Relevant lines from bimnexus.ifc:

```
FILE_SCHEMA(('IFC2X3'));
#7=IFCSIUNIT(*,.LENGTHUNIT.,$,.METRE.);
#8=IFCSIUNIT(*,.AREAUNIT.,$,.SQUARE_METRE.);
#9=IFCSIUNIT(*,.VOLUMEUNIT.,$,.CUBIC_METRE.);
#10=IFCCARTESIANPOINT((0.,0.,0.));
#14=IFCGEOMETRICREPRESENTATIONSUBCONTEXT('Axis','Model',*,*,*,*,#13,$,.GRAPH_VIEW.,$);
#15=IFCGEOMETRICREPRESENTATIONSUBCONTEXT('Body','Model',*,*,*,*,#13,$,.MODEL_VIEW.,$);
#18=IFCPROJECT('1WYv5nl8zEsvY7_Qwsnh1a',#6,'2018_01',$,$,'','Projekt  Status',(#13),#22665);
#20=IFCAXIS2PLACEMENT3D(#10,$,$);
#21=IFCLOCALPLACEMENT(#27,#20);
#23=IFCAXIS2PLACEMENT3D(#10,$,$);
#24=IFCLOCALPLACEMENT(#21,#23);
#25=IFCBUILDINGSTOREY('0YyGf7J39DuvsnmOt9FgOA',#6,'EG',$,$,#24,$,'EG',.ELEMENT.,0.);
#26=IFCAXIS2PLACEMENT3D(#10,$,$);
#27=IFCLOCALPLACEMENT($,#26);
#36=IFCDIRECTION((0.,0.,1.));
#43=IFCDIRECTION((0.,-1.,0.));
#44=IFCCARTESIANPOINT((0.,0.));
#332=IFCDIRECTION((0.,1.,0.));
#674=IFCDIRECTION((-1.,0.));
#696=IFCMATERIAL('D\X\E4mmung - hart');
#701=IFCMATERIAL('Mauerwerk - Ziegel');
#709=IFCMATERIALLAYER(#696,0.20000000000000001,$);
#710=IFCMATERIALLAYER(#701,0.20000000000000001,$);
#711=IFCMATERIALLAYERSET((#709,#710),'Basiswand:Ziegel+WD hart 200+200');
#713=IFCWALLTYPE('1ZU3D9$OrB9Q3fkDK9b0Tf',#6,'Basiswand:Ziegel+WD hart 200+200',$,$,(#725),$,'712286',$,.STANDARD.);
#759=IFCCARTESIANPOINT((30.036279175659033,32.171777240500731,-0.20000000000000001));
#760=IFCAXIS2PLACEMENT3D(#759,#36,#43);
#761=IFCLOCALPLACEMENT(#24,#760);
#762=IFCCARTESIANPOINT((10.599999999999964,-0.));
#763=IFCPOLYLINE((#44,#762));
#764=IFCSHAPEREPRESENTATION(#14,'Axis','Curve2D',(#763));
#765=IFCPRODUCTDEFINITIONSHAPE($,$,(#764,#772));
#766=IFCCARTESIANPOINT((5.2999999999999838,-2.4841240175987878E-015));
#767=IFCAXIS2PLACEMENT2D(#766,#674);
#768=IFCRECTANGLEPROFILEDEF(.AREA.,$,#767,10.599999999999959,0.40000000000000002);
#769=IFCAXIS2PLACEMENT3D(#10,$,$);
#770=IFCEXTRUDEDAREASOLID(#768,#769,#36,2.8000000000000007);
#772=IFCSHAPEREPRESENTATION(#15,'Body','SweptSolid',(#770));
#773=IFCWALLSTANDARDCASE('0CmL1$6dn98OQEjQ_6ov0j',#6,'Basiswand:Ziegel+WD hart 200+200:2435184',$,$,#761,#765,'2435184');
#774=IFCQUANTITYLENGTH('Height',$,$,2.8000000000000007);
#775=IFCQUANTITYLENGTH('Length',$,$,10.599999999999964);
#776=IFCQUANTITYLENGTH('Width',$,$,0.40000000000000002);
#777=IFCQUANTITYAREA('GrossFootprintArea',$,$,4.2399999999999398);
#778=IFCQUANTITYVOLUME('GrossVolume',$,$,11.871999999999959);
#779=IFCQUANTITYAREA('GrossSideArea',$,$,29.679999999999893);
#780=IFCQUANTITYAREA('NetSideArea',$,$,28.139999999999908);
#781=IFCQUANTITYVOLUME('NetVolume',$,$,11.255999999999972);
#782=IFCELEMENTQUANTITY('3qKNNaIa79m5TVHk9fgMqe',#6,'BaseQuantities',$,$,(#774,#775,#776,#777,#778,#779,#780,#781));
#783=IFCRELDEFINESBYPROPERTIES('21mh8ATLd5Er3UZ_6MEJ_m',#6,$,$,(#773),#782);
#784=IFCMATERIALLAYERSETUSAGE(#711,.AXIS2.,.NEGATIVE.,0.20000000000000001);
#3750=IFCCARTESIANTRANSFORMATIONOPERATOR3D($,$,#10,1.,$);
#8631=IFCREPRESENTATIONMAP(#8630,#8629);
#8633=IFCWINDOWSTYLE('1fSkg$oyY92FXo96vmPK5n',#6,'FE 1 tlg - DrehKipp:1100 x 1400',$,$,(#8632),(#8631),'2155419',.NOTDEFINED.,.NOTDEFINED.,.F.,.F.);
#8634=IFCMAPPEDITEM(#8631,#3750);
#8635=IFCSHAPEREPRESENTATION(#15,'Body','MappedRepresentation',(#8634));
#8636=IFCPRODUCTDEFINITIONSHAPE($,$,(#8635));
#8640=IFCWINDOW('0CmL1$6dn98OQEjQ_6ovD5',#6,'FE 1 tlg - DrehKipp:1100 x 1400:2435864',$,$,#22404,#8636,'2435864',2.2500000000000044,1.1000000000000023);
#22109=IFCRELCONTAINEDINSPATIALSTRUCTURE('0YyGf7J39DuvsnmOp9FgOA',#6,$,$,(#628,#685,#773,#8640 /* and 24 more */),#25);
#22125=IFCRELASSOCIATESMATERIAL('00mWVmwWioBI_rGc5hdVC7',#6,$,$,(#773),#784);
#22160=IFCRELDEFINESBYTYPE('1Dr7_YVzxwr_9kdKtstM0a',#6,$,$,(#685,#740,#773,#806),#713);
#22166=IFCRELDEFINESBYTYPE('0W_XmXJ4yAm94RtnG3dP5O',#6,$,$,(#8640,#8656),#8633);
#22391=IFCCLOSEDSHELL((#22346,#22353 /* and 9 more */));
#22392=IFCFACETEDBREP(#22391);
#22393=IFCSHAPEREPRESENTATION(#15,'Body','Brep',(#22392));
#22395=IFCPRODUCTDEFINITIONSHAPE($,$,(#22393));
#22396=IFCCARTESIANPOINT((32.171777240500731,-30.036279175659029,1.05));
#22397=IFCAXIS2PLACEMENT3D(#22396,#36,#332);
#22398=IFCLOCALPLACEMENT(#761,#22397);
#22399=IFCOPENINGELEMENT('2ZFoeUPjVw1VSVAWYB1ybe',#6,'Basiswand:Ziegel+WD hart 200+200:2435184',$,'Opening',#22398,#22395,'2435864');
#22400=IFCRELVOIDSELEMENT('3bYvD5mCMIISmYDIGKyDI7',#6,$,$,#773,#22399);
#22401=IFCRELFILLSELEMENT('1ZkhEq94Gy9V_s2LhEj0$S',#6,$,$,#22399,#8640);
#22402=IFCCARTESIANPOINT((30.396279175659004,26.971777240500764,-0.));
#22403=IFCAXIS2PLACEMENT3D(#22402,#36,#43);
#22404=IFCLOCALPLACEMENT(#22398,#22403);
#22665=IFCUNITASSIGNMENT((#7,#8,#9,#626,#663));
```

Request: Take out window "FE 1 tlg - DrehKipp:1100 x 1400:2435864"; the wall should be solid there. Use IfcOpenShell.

```python
import ifcopenshell
import ifcopenshell.api.feature
import ifcopenshell.api.pset
import ifcopenshell.api.root
import ifcopenshell.geom
import ifcopenshell.util.element
import ifcopenshell.util.shape
import ifcopenshell.util.unit

model = ifcopenshell.open("bimnexus.ifc")
area_scale = ifcopenshell.util.unit.calculate_unit_scale(model, "AREAUNIT")
volume_scale = ifcopenshell.util.unit.calculate_unit_scale(model, "VOLUMEUNIT")
settings = ifcopenshell.geom.settings()


def volume(element):
    """Net volume in cubic metres, openings subtracted."""
    shape = ifcopenshell.geom.create_shape(settings, element)
    return ifcopenshell.util.shape.get_volume(shape.geometry)


window = model.by_guid("0CmL1$6dn98OQEjQ_6ovD5")
opening = window.FillsVoids[0].RelatingOpeningElement
wall = opening.VoidsElements[0].RelatingBuildingElement
before = volume(wall)

ifcopenshell.api.root.remove_product(model, product=window)
ifcopenshell.api.feature.remove_feature(model, feature=opening)

after = volume(wall)
thickness = 0.4  # wall thickness in metres

# Update the wall's stored quantities.
qto = model.by_id(ifcopenshell.util.element.get_pset(wall, "BaseQuantities", should_inherit=False)["id"])
ifcopenshell.api.pset.edit_qto(model, qto=qto, properties={
    "NetSideArea": after / thickness / area_scale,
    "NetVolume": after / volume_scale,
})

print(f"wall volume {before:.3f} -> {after:.3f} m3")

model.write("bimnexus_v2.ifc")
```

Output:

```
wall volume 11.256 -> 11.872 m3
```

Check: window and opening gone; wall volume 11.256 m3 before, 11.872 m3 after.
